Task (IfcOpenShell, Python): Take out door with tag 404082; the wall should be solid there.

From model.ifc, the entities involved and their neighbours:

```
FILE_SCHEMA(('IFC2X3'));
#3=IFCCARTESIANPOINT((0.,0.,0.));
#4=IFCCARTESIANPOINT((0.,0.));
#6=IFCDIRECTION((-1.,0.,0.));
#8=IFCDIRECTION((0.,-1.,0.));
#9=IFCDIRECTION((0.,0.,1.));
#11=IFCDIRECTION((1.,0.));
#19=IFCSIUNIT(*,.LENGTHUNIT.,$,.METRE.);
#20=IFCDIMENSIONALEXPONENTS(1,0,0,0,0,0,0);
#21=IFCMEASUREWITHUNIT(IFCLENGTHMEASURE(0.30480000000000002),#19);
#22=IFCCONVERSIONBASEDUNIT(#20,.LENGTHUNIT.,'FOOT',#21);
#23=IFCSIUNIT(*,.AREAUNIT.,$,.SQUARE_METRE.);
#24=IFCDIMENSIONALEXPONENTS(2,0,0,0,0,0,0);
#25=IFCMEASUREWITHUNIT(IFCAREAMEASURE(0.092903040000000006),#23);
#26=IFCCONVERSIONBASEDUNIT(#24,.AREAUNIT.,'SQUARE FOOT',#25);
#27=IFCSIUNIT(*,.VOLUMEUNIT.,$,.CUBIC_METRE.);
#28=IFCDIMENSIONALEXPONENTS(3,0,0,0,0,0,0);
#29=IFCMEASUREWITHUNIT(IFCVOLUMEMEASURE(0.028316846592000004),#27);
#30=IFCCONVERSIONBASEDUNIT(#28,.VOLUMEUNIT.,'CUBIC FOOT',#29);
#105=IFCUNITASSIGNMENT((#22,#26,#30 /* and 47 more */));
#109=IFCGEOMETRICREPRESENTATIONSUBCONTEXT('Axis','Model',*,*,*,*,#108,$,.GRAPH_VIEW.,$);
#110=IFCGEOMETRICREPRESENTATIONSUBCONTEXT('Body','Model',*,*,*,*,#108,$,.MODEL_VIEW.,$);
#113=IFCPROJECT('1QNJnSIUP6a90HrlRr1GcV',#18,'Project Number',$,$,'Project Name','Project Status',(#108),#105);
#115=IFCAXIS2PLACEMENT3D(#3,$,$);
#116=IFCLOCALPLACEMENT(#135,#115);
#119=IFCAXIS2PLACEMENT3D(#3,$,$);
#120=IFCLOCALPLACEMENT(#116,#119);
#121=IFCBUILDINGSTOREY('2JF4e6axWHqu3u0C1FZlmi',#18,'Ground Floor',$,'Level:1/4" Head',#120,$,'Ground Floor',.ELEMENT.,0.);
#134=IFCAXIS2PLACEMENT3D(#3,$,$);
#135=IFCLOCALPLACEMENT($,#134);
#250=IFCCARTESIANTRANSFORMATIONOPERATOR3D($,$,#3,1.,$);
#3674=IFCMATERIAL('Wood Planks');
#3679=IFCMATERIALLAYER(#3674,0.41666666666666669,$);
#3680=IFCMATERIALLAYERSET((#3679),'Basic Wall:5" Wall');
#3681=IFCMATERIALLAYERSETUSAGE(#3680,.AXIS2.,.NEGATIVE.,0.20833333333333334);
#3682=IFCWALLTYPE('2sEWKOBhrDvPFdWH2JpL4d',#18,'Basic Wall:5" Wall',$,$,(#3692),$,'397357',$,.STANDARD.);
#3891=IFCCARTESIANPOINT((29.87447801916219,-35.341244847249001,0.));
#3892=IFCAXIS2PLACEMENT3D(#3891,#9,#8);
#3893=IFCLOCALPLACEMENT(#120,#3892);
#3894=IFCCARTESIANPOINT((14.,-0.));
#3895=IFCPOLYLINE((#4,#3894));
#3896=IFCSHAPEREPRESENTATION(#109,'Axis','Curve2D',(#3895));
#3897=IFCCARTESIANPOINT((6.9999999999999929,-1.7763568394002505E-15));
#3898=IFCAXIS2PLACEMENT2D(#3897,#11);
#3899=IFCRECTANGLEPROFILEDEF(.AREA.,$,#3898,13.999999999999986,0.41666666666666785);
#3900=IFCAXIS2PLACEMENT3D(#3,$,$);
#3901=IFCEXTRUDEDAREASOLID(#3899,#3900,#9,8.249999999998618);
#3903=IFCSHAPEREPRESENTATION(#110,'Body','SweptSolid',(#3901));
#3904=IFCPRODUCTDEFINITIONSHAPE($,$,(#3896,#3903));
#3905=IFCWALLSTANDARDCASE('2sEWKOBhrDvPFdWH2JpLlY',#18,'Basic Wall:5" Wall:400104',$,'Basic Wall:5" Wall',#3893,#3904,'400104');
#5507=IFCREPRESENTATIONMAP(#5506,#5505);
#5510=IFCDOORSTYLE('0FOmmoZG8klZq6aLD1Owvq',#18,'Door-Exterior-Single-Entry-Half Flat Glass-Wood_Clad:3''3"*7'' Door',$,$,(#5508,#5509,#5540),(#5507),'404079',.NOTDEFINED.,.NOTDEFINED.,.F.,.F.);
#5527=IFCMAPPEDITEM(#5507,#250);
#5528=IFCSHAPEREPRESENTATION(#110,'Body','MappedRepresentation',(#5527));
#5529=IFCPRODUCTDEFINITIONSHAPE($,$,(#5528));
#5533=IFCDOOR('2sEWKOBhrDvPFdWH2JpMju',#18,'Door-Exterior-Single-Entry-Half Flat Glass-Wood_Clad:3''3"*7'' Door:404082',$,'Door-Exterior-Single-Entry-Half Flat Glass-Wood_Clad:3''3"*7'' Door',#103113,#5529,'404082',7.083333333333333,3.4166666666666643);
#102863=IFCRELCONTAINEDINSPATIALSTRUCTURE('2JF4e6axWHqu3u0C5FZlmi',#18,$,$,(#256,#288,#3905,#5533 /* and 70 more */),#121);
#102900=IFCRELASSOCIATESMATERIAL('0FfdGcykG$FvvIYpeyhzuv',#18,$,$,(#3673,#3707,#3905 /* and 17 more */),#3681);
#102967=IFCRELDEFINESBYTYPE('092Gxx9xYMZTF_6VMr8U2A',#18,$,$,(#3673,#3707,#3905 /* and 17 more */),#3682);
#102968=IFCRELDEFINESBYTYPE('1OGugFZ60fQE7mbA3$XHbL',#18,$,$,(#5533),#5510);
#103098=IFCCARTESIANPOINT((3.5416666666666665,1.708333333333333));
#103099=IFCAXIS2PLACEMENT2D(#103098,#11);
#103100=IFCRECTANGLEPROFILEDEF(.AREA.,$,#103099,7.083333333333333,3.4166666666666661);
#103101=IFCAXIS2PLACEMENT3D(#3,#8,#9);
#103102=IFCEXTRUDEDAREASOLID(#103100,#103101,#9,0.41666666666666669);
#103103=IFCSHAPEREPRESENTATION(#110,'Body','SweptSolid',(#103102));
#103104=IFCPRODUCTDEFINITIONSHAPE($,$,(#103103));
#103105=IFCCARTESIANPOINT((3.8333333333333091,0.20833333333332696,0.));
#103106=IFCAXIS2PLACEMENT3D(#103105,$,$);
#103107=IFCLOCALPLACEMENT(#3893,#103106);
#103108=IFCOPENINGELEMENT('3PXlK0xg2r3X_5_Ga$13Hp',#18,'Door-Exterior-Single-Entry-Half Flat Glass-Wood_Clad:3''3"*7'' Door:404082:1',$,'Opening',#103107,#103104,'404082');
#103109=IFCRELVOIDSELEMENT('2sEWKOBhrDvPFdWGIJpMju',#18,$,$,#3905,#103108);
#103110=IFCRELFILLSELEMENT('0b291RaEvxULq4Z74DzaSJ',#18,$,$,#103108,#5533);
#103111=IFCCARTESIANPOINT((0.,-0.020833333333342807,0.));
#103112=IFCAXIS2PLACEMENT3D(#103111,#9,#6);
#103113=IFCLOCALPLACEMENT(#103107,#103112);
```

```python
import ifcopenshell
import ifcopenshell.api.feature
import ifcopenshell.api.root
import ifcopenshell.geom
import ifcopenshell.util.shape

model = ifcopenshell.open("model.ifc")
settings = ifcopenshell.geom.settings()


def volume(element):
    """Net volume in cubic metres, openings subtracted."""
    shape = ifcopenshell.geom.create_shape(settings, element)
    return ifcopenshell.util.shape.get_volume(shape.geometry)


door = model.by_guid("2sEWKOBhrDvPFdWH2JpMju")
opening = door.FillsVoids[0].RelatingOpeningElement
wall = opening.VoidsElements[0].RelatingBuildingElement
before = volume(wall)

ifcopenshell.api.root.remove_product(model, product=door)
ifcopenshell.api.feature.remove_feature(model, feature=opening)

after = volume(wall)

print(f"wall volume {before:.3f} -> {after:.3f} m3")

model.write("model_v2.ifc")
```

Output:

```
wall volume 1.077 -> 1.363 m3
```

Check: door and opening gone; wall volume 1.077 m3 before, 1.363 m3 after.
